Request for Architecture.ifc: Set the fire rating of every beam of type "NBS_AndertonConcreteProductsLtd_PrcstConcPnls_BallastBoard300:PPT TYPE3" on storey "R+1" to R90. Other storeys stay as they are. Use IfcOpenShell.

First a look at what the model holds.

```python
import ifcopenshell
import ifcopenshell.util.element

model = ifcopenshell.open("Architecture.ifc")
print(model.schema)
storey = next(s for s in model.by_type("IfcBuildingStorey") if s.Name == "R+1")
beams = [e for e in ifcopenshell.util.element.get_decomposition(storey) if e.is_a("IfcBeam")]
seen = {}
for e in beams:
    element_type = ifcopenshell.util.element.get_type(e)
    key = (element_type.Name if element_type != e and element_type else None, ifcopenshell.util.element.get_pset(e, "Pset_BeamCommon", "FireRating"))
    seen[key] = seen.get(key, 0) + 1
for (name, value), count in sorted(seen.items(), key=str):
    print(count, "x", name, "|", value)
```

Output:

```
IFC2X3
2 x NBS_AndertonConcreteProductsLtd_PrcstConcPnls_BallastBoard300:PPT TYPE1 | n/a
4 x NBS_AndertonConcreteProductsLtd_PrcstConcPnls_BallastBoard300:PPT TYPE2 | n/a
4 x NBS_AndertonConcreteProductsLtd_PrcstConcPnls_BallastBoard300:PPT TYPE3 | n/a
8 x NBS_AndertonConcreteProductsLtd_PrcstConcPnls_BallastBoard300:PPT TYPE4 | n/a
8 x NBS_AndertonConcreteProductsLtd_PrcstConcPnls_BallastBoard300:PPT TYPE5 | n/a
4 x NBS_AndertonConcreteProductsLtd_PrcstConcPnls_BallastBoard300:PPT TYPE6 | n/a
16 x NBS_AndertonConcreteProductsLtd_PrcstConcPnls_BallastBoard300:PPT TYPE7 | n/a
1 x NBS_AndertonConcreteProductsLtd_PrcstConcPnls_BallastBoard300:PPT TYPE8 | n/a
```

```python
import ifcopenshell
import ifcopenshell.api.pset
import ifcopenshell.util.element

model = ifcopenshell.open("Architecture.ifc")

storey = next(s for s in model.by_type("IfcBuildingStorey") if s.Name == "R+1")
beams = [e for e in ifcopenshell.util.element.get_decomposition(storey) if e.is_a("IfcBeam")]

count = 0
for e in beams:
    element_type = ifcopenshell.util.element.get_type(e)
    if element_type in (None, e) or element_type.Name != "NBS_AndertonConcreteProductsLtd_PrcstConcPnls_BallastBoard300:PPT TYPE3":
        continue
    # add_pset returns the element's existing set when there is one.
    pset = ifcopenshell.api.pset.add_pset(model, product=e, name="Pset_BeamCommon")
    ifcopenshell.api.pset.edit_pset(model, pset=pset, properties={"FireRating": "R90"})
    count += 1

print(count, "beams updated")

model.write("Architecture_v2.ifc")
```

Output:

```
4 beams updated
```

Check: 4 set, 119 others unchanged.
